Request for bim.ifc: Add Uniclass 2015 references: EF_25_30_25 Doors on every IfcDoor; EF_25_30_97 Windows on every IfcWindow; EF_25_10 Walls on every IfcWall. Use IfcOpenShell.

First a look at what the model holds.

```python
import ifcopenshell

model = ifcopenshell.open("bim.ifc")
print(model.schema)
print("classifications:", [c.Name for c in model.by_type("IfcClassification")])
for ifc_class in ("IfcDoor", "IfcRoof", "IfcStair", "IfcWall", "IfcWindow"):
    print(ifc_class, len(model.by_type(ifc_class)))
```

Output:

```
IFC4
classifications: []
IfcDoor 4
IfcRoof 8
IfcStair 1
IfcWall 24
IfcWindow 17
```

```python
import ifcopenshell
import ifcopenshell.api.classification

model = ifcopenshell.open("bim.ifc")

system = ifcopenshell.api.classification.add_classification(model, classification="Uniclass 2015")

codes = {
    "IfcDoor": ("EF_25_30_25", "Doors"),
    "IfcWindow": ("EF_25_30_97", "Windows"),
    "IfcWall": ("EF_25_10", "Walls"),
}
for ifc_class, (code, name) in codes.items():
    products = model.by_type(ifc_class)
    ifcopenshell.api.classification.add_reference(
        model, products=products, classification=system, identification=code, name=name
    )
    print(code, len(products))

model.write("bim-out.ifc")
```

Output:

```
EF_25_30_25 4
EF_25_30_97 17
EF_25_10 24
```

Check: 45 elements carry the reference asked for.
